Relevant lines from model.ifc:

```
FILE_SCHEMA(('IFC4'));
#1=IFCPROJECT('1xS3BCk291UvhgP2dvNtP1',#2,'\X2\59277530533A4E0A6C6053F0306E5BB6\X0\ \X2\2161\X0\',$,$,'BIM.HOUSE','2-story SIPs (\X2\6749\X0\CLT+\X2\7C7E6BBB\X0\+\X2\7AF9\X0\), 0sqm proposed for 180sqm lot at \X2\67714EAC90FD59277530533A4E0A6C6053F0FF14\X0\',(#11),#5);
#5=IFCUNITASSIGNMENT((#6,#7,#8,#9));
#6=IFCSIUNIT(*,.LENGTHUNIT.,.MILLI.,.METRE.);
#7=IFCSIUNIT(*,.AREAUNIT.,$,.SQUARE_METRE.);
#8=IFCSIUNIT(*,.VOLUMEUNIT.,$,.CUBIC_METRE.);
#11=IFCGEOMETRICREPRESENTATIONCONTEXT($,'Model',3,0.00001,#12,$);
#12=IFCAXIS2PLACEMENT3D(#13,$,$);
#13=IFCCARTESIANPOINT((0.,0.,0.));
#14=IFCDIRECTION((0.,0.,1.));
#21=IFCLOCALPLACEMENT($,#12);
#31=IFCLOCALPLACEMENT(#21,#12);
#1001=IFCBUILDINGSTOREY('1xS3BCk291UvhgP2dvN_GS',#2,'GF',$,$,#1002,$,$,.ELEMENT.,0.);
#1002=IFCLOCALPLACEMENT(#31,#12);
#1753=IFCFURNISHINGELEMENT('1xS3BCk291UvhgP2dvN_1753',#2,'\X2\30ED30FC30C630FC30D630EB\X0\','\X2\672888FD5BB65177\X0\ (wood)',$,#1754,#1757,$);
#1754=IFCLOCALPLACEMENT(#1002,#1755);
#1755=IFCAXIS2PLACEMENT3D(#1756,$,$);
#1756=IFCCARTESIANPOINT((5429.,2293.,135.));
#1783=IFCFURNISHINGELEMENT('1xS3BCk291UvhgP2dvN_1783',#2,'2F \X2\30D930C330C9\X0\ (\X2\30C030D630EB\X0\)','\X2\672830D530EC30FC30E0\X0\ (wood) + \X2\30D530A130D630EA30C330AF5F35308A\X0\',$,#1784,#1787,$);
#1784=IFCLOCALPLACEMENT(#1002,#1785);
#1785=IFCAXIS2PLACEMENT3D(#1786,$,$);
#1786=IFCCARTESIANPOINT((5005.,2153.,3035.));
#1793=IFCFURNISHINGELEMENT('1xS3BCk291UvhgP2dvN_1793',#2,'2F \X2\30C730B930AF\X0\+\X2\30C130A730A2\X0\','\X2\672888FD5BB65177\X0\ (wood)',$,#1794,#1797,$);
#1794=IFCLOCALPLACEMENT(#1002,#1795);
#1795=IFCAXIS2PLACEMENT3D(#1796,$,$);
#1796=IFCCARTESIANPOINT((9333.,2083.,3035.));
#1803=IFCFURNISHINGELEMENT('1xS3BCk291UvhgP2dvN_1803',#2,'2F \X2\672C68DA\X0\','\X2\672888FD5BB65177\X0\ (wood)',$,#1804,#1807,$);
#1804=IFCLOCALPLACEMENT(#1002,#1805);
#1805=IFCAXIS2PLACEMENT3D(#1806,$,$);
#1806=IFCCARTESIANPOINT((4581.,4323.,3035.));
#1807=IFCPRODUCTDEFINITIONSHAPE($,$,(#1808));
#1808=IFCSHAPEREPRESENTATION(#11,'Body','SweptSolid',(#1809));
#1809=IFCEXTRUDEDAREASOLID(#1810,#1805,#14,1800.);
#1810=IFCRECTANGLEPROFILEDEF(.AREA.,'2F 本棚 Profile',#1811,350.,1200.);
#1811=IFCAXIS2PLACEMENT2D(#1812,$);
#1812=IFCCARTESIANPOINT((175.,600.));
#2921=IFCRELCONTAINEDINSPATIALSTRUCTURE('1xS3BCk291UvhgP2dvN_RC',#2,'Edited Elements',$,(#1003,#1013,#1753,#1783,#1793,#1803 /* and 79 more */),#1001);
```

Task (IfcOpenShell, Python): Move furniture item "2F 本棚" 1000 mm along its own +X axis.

```python
import ifcopenshell
import ifcopenshell.api.geometry
import ifcopenshell.util.placement
import ifcopenshell.util.unit

model = ifcopenshell.open("model.ifc")
unit_scale = ifcopenshell.util.unit.calculate_unit_scale(model)

item = model.by_id(1803)
matrix = ifcopenshell.util.placement.get_local_placement(item.ObjectPlacement)
matrix[:3, 3] += matrix[:3, 0] * 1 / unit_scale
ifcopenshell.api.geometry.edit_object_placement(model, product=item, matrix=matrix, is_si=False)

print(ifcopenshell.util.placement.get_local_placement(item.ObjectPlacement).round(3) + 0.0)

model.write("model_edited.ifc")
```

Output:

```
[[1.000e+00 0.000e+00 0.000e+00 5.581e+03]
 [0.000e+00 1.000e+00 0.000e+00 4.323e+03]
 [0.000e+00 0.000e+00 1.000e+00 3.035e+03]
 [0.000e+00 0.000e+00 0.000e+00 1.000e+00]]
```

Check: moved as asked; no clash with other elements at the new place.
